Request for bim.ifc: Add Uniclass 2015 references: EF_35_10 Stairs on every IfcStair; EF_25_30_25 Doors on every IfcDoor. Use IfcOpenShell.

First a look at what the model holds.

```python
import ifcopenshell

model = ifcopenshell.open("bim.ifc")
print(model.schema)
print("classifications:", [c.Name for c in model.by_type("IfcClassification")])
for ifc_class in ("IfcDoor", "IfcRoof", "IfcStair", "IfcWall", "IfcWindow"):
    print(ifc_class, len(model.by_type(ifc_class)))
```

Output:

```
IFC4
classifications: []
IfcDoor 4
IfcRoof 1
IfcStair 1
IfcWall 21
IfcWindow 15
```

```python
import ifcopenshell
import ifcopenshell.api.classification

model = ifcopenshell.open("bim.ifc")

system = ifcopenshell.api.classification.add_classification(model, classification="Uniclass 2015")

codes = {
    "IfcStair": ("EF_35_10", "Stairs"),
    "IfcDoor": ("EF_25_30_25", "Doors"),
}
for ifc_class, (code, name) in codes.items():
    products = model.by_type(ifc_class)
    ifcopenshell.api.classification.add_reference(
        model, products=products, classification=system, identification=code, name=name
    )
    print(code, len(products))

model.write("bim_v2.ifc")
```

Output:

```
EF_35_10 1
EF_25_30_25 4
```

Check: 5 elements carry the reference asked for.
